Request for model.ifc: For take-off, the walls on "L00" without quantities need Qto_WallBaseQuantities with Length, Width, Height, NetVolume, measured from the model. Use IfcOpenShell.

First a look at what the model holds.

```python
import ifcopenshell
import ifcopenshell.util.element
import ifcopenshell.util.unit

model = ifcopenshell.open("model.ifc")
print(model.schema)
for unit_type in ("LENGTHUNIT", "AREAUNIT", "VOLUMEUNIT"):
    print(unit_type, ifcopenshell.util.unit.calculate_unit_scale(model, unit_type))
storey = next(s for s in model.by_type("IfcBuildingStorey") if s.Name == "L00")
walls = [e for e in ifcopenshell.util.element.get_decomposition(storey) if e.is_a("IfcWall")]
for e in sorted(walls, key=lambda e: e.id()):
    print(e.id(), e.is_a(), e.Name, list(ifcopenshell.util.element.get_psets(e, qtos_only=True)), sep=" | ")
```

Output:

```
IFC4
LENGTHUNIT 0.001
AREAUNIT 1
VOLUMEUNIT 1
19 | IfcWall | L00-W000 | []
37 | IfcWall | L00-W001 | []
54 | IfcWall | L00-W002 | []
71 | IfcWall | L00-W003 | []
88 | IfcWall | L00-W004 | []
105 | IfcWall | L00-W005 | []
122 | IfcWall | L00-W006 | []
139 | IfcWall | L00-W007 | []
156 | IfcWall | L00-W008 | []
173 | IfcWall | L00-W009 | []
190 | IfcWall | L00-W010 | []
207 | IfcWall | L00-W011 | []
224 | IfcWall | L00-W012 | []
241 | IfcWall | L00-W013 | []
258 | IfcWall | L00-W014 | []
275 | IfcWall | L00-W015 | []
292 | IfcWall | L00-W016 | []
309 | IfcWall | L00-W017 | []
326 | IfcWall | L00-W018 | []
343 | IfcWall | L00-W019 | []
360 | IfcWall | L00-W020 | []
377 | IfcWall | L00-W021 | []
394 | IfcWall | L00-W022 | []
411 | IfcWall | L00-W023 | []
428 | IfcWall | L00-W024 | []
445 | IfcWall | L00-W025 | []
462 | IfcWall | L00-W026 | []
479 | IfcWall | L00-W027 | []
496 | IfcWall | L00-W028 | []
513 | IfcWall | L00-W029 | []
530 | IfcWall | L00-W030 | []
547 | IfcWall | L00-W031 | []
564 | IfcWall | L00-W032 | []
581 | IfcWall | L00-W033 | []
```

```python
import ifcopenshell
import ifcopenshell.api.pset
import ifcopenshell.geom
import ifcopenshell.util.element
import ifcopenshell.util.shape
import ifcopenshell.util.unit

model = ifcopenshell.open("model.ifc")
unit_scale = ifcopenshell.util.unit.calculate_unit_scale(model)
volume_scale = ifcopenshell.util.unit.calculate_unit_scale(model, "VOLUMEUNIT")
settings = ifcopenshell.geom.settings()

storey = next(s for s in model.by_type("IfcBuildingStorey") if s.Name == "L00")
walls = [e for e in ifcopenshell.util.element.get_decomposition(storey) if e.is_a("IfcWall")]

for e in sorted(walls, key=lambda e: e.id()):
    if ifcopenshell.util.element.get_psets(e, qtos_only=True, should_inherit=False):
        continue
    # Geometry comes back in metres, in the element's own axes.
    shape = ifcopenshell.geom.create_shape(settings, e)
    values = {
        "Length": ifcopenshell.util.shape.get_x(shape.geometry) / unit_scale,
        "Width": ifcopenshell.util.shape.get_y(shape.geometry) / unit_scale,
        "Height": ifcopenshell.util.shape.get_z(shape.geometry) / unit_scale,
        "NetVolume": ifcopenshell.util.shape.get_volume(shape.geometry) / volume_scale,
    }
    qto = ifcopenshell.api.pset.add_qto(model, product=e, name="Qto_WallBaseQuantities")
    ifcopenshell.api.pset.edit_qto(model, qto=qto, properties=values)
    print(e.id(), {k: round(v, 3) for k, v in values.items()})

model.write("model-out.ifc")
```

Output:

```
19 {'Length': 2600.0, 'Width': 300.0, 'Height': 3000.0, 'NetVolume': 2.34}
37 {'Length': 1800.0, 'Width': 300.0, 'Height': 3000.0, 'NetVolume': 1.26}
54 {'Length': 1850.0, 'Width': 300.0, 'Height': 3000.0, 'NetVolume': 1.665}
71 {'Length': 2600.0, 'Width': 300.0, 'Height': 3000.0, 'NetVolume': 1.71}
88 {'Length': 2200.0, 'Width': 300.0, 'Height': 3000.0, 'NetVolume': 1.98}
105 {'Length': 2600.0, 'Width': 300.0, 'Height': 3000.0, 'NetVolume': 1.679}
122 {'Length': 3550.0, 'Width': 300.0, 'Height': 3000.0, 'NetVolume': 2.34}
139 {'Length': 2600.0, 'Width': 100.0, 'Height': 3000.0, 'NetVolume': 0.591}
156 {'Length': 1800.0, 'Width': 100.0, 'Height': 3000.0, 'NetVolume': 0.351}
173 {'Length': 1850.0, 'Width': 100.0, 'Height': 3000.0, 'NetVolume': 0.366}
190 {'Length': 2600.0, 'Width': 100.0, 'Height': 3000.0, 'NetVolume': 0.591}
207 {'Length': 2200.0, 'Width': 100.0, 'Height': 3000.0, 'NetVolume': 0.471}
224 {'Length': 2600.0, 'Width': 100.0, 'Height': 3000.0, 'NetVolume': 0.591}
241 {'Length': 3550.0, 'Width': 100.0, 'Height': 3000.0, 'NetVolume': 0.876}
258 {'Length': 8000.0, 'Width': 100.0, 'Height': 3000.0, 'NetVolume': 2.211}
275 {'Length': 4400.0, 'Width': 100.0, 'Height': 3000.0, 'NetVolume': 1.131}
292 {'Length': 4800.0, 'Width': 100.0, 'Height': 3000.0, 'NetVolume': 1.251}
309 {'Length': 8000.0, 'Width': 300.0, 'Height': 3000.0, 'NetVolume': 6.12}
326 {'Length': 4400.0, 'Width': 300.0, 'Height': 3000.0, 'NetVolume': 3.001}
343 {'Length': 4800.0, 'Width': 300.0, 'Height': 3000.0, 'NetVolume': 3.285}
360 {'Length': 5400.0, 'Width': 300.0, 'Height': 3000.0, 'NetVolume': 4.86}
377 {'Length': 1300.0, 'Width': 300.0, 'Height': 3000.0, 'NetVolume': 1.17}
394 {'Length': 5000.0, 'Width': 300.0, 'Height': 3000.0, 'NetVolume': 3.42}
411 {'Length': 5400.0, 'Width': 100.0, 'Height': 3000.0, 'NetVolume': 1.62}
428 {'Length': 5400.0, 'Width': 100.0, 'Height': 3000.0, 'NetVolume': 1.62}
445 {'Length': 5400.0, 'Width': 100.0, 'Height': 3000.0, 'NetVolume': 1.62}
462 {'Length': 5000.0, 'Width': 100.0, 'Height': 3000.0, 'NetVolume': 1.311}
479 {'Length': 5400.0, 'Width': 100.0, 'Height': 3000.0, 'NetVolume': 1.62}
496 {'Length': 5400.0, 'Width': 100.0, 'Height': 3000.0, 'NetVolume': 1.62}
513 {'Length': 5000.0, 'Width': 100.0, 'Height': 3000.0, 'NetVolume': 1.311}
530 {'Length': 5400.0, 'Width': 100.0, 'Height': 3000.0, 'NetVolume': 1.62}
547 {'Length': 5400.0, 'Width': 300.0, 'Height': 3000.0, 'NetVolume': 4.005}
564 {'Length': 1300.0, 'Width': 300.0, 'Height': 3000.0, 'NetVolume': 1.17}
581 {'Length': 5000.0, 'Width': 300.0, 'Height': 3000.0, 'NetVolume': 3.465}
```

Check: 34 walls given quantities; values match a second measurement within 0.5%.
